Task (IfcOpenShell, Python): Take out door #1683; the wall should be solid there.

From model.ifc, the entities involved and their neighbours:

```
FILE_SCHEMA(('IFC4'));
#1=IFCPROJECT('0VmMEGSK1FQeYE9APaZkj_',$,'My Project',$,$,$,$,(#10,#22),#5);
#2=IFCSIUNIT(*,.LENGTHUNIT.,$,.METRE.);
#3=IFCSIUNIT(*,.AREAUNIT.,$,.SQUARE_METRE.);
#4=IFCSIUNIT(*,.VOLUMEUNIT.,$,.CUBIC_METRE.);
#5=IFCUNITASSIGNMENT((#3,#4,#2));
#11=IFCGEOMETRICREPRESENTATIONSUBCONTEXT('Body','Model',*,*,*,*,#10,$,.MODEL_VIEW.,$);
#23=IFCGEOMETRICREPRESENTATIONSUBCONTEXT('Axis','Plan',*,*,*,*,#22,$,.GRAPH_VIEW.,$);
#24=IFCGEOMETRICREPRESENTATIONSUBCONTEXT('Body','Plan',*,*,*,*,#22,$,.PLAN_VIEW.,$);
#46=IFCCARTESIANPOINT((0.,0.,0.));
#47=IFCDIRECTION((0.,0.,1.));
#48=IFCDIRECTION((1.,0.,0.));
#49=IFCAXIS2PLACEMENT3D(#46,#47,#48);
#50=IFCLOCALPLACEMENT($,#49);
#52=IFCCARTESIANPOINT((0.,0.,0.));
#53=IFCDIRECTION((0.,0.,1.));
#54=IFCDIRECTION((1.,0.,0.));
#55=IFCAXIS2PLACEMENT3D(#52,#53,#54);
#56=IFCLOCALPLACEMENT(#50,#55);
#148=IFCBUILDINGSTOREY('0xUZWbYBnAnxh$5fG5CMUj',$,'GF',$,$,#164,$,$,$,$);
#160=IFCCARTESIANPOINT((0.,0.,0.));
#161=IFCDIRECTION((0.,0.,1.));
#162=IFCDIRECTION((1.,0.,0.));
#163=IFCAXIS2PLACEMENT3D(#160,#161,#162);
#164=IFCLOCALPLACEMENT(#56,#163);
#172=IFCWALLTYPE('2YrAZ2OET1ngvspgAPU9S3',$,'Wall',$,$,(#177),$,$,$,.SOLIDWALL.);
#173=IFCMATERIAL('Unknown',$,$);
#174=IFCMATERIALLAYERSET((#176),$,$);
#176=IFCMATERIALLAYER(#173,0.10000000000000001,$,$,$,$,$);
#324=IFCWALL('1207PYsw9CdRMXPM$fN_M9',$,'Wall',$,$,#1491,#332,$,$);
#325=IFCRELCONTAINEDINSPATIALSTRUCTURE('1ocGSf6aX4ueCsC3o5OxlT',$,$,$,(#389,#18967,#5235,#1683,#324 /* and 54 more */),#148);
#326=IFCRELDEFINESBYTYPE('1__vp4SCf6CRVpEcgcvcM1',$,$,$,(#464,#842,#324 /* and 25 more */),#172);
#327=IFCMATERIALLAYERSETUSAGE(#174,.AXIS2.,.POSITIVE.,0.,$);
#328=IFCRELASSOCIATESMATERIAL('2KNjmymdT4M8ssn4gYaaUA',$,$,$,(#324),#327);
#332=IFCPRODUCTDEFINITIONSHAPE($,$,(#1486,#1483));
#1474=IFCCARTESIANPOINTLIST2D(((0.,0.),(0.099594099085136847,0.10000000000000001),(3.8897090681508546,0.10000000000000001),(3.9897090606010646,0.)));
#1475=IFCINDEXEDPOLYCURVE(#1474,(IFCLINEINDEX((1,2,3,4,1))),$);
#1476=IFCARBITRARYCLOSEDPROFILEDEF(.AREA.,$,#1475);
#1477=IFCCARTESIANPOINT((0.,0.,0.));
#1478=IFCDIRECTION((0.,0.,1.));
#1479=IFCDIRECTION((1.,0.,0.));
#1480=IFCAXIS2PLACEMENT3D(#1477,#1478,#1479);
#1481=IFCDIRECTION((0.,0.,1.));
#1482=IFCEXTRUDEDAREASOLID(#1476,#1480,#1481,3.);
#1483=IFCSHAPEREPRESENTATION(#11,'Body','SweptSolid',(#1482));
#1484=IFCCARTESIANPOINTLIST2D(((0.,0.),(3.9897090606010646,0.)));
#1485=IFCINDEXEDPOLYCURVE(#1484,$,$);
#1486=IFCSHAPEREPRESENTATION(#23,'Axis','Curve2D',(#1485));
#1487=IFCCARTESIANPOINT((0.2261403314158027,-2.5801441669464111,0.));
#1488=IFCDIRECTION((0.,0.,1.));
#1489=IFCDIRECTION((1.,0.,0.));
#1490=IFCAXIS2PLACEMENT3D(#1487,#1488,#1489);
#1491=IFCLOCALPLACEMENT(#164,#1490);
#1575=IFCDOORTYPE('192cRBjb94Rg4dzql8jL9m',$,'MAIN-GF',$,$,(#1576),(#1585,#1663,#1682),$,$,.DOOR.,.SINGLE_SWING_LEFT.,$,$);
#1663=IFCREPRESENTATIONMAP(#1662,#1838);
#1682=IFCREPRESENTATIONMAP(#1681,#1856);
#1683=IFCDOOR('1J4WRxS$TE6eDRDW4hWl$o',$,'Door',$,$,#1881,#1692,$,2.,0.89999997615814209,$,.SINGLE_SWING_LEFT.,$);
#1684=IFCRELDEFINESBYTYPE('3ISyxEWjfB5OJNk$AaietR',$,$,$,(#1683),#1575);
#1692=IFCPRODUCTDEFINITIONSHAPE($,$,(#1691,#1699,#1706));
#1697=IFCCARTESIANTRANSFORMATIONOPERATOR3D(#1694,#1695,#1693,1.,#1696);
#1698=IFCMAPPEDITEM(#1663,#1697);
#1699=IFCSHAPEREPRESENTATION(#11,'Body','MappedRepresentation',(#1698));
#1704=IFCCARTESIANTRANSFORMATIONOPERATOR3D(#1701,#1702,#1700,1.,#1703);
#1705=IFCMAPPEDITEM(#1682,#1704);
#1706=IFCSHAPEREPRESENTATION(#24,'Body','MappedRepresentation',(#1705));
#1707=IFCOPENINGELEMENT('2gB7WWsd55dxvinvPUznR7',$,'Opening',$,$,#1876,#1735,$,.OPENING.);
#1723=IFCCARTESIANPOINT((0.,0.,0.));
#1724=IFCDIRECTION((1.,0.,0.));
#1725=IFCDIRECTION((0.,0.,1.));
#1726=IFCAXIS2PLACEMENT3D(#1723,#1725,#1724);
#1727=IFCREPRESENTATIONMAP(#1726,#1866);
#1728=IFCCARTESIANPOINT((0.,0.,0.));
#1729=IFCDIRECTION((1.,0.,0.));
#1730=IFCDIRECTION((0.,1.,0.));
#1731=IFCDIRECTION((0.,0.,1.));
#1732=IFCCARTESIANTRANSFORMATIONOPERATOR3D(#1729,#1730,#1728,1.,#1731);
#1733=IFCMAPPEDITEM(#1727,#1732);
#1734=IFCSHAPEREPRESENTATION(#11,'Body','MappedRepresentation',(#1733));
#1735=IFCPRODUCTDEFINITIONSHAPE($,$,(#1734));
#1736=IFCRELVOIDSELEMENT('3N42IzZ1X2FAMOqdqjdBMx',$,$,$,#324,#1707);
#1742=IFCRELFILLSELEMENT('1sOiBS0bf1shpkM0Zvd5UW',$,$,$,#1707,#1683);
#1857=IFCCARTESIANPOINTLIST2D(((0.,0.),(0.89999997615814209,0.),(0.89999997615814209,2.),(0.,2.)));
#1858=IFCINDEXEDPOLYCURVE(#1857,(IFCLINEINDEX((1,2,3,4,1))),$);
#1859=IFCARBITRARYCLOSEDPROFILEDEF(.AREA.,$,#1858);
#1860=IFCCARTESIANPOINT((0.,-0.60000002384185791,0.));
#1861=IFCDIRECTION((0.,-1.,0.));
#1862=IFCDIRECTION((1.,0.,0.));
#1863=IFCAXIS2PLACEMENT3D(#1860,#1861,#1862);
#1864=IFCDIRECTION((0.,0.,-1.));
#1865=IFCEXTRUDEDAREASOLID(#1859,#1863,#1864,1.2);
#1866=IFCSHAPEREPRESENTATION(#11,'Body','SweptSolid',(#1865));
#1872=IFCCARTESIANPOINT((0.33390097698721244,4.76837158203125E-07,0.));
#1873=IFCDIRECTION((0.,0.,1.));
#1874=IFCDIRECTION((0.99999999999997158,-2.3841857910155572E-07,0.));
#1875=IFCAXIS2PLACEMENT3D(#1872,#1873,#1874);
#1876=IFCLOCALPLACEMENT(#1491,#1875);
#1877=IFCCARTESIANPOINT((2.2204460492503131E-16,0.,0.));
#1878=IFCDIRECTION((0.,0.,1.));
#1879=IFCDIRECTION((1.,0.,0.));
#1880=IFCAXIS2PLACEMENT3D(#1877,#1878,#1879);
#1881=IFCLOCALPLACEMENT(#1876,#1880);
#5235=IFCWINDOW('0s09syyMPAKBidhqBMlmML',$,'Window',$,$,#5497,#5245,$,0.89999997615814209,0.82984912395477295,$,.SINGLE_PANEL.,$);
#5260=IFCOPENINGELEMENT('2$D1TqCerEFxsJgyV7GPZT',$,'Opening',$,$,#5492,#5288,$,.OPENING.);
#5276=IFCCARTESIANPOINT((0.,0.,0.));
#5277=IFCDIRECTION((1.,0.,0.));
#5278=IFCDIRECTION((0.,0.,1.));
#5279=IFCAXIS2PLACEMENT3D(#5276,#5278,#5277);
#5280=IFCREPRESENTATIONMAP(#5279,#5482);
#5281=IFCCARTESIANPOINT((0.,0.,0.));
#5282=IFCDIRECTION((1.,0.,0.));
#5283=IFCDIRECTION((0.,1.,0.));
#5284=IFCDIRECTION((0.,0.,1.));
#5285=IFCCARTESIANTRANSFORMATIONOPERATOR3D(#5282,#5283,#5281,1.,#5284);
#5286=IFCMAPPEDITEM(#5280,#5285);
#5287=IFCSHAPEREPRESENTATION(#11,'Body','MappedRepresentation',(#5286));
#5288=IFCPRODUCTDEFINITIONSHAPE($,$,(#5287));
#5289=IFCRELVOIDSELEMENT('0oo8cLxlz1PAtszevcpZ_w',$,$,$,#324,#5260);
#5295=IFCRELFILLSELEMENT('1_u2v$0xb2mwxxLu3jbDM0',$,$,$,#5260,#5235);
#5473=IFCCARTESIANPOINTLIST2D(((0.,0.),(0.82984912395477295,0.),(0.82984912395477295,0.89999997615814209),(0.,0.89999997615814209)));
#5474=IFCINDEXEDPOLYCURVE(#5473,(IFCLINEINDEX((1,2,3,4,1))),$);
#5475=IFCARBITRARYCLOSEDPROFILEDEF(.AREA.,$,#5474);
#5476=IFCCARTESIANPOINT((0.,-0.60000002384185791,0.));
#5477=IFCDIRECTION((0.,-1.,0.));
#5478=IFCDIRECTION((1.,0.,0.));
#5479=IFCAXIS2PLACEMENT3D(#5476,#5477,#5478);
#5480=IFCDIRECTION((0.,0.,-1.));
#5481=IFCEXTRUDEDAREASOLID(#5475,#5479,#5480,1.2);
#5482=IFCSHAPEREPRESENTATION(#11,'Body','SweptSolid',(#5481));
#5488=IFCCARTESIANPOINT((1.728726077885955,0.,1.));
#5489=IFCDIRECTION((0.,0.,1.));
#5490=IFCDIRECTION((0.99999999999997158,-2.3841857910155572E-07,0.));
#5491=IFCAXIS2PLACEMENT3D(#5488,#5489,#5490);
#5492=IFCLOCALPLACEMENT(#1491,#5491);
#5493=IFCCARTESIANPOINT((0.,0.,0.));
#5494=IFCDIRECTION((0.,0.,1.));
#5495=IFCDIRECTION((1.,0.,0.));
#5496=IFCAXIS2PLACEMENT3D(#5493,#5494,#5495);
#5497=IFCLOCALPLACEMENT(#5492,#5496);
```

```python
import ifcopenshell
import ifcopenshell.api.feature
import ifcopenshell.api.root
import ifcopenshell.geom
import ifcopenshell.util.shape

model = ifcopenshell.open("model.ifc")
settings = ifcopenshell.geom.settings()


def volume(element):
    """Net volume in cubic metres, openings subtracted."""
    shape = ifcopenshell.geom.create_shape(settings, element)
    return ifcopenshell.util.shape.get_volume(shape.geometry)


door = model.by_guid("1J4WRxS$TE6eDRDW4hWl$o")
opening = door.FillsVoids[0].RelatingOpeningElement
wall = opening.VoidsElements[0].RelatingBuildingElement
before = volume(wall)

ifcopenshell.api.root.remove_product(model, product=door)
ifcopenshell.api.feature.remove_feature(model, feature=opening)

after = volume(wall)

print(f"wall volume {before:.3f} -> {after:.3f} m3")

model.write("model_v2.ifc")
```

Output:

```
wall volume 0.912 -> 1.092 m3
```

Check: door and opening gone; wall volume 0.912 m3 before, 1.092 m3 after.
